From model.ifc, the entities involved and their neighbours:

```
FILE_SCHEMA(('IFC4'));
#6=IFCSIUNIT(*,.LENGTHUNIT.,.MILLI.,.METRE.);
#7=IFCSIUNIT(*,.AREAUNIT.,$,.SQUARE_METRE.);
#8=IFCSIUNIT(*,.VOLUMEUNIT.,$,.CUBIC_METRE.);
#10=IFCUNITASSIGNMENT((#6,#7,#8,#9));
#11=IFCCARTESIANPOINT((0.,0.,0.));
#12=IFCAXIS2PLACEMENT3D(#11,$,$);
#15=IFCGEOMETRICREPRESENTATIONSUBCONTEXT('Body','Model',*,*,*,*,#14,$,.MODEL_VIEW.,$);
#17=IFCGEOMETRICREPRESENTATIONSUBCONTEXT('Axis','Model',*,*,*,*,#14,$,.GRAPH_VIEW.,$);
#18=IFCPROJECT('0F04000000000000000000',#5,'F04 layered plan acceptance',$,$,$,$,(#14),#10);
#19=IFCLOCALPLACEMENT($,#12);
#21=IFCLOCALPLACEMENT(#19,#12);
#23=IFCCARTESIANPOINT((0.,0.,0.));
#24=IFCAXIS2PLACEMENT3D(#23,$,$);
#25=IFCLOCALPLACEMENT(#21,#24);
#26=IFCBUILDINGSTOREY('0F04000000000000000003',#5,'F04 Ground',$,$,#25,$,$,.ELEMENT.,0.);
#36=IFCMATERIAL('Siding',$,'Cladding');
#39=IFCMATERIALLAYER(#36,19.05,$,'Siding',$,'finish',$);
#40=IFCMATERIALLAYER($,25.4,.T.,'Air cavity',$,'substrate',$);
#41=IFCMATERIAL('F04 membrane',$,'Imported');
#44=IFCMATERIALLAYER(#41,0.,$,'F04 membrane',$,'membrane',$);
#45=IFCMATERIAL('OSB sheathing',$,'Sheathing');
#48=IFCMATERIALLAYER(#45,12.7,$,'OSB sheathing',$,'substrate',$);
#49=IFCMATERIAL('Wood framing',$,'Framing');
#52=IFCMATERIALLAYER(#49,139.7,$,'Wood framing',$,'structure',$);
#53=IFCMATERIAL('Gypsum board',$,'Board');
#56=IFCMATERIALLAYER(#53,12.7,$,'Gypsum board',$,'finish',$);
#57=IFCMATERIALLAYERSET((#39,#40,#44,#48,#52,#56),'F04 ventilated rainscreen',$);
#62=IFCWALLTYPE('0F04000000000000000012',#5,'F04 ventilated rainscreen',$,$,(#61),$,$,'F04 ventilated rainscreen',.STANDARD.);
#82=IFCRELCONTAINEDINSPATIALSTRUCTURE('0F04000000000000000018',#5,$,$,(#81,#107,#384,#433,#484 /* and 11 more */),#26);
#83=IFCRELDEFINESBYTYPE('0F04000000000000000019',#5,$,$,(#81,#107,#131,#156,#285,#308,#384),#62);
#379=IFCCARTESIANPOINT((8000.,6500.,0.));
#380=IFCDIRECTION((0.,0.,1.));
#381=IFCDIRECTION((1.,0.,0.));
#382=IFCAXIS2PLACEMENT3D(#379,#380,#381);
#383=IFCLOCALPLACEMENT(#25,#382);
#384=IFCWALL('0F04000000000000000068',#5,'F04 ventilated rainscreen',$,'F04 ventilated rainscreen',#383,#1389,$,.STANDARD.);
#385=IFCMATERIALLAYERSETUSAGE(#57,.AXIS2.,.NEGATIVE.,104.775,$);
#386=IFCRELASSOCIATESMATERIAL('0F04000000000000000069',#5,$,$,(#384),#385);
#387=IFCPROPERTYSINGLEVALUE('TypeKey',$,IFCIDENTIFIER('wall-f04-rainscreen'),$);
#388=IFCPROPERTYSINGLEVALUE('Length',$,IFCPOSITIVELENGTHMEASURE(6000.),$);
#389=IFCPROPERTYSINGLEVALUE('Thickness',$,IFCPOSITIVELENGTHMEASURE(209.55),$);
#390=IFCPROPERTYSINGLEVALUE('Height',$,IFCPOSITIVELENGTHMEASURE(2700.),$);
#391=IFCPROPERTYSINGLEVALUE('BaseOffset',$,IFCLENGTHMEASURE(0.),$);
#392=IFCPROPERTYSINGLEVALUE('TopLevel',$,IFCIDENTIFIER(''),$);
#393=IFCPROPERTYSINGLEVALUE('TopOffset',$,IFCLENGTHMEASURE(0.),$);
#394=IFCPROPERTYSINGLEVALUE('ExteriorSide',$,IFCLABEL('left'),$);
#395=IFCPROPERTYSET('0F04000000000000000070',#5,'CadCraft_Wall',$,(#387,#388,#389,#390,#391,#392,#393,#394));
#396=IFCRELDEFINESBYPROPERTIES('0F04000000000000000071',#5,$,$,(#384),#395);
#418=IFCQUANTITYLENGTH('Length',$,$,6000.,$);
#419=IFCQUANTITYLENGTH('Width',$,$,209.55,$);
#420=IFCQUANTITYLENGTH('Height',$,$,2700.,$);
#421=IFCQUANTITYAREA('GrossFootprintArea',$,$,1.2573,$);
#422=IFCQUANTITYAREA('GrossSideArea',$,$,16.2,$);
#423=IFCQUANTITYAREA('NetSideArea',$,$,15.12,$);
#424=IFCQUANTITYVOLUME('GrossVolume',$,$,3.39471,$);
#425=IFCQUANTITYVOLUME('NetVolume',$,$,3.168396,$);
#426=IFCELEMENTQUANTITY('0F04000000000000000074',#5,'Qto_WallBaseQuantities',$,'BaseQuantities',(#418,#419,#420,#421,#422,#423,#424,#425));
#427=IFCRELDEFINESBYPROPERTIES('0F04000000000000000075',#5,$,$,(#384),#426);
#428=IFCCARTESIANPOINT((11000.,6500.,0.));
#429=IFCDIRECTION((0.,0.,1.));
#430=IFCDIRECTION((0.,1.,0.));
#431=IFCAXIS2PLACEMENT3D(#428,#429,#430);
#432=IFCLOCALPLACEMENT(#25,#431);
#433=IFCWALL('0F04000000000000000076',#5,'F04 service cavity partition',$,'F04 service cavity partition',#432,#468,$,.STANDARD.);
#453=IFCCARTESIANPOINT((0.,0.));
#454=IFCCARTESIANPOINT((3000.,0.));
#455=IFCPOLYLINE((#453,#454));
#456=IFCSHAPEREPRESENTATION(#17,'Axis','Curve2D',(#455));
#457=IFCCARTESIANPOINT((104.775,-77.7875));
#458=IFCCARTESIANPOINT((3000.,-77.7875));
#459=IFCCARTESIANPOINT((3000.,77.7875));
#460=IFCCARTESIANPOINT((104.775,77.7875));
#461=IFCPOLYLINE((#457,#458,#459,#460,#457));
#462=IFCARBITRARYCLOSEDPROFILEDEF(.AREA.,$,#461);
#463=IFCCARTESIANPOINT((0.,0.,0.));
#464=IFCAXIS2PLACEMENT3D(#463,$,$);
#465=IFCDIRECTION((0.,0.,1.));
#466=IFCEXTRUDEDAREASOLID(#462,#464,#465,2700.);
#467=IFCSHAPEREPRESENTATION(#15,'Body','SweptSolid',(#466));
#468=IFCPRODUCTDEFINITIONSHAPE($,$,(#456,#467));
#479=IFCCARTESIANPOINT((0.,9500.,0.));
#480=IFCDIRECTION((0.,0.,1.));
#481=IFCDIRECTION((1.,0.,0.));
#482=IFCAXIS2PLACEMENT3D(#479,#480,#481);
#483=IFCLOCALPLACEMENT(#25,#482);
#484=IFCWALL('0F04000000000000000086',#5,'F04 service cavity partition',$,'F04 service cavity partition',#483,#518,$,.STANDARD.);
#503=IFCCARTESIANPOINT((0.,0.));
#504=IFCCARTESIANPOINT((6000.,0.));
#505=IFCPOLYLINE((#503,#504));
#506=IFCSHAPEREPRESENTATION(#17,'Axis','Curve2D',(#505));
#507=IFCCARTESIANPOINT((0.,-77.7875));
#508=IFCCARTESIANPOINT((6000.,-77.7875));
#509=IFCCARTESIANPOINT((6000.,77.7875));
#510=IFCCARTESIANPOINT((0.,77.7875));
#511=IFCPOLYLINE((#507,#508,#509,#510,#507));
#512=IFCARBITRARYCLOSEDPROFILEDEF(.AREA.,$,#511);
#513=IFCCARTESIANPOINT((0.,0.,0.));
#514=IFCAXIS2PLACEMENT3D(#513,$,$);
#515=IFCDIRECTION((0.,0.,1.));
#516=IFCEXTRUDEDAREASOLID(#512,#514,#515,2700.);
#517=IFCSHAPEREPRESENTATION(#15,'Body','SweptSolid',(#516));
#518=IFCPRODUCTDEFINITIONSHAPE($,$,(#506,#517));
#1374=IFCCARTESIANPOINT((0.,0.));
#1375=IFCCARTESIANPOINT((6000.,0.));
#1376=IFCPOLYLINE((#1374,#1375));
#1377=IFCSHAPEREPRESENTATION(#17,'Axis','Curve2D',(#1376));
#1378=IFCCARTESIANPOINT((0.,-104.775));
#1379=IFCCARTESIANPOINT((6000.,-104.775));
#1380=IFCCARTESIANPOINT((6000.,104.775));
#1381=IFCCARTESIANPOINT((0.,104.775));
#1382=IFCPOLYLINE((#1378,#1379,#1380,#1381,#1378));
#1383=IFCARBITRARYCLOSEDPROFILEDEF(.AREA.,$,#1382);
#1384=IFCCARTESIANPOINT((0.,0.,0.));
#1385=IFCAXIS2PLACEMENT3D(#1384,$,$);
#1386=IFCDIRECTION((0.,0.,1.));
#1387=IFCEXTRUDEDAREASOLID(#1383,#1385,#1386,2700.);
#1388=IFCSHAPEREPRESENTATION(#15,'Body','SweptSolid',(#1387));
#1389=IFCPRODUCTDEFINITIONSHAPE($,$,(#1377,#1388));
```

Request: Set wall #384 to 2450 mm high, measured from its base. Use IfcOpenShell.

```python
import ifcopenshell
import ifcopenshell.api.pset
import ifcopenshell.geom
import ifcopenshell.util.element
import ifcopenshell.util.representation
import ifcopenshell.util.shape
import ifcopenshell.util.unit

model = ifcopenshell.open("model.ifc")
unit_scale = ifcopenshell.util.unit.calculate_unit_scale(model)
area_scale = ifcopenshell.util.unit.calculate_unit_scale(model, "AREAUNIT")
volume_scale = ifcopenshell.util.unit.calculate_unit_scale(model, "VOLUMEUNIT")
settings = ifcopenshell.geom.settings()


def volume(element):
    """Net volume in cubic metres, openings subtracted."""
    shape = ifcopenshell.geom.create_shape(settings, element)
    return ifcopenshell.util.shape.get_volume(shape.geometry)


wall = model.by_guid("0F04000000000000000068")
before = volume(wall)

body = ifcopenshell.util.representation.get_representation(wall, "Model", "Body")
solid = body.Items[0]
old_height = solid.Depth
solid.Depth = 2450.0
after = volume(wall)
thickness = 0.2096  # wall thickness in metres

# Update the stored height, areas and volumes.
pset = model.by_id(ifcopenshell.util.element.get_pset(wall, "CadCraft_Wall", should_inherit=False)["id"])
ifcopenshell.api.pset.edit_pset(model, pset=pset, properties={
    "Height": model.create_entity("IfcPositiveLengthMeasure", solid.Depth),
})
qto = model.by_id(ifcopenshell.util.element.get_pset(wall, "Qto_WallBaseQuantities", should_inherit=False)["id"])
ifcopenshell.api.pset.edit_qto(model, qto=qto, properties={
    "Height": solid.Depth,
    "GrossSideArea": ifcopenshell.util.element.get_pset(wall, "Qto_WallBaseQuantities", "GrossSideArea") * solid.Depth / old_height,
    "NetSideArea": after / thickness / area_scale,
    "GrossVolume": ifcopenshell.util.element.get_pset(wall, "Qto_WallBaseQuantities", "GrossVolume") * solid.Depth / old_height,
    "NetVolume": after / volume_scale,
})

print(f"height {old_height:g} -> {solid.Depth:g}, volume {before:.3f} -> {after:.3f} m3")

model.write("model_rev.ifc")
```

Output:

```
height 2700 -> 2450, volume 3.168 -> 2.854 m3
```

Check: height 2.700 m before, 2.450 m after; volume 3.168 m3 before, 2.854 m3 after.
